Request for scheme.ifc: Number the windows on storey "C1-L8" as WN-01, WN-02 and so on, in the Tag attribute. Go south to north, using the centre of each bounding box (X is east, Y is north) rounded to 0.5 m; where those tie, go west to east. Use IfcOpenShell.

First a look at what the model holds.

```python
import ifcopenshell
import ifcopenshell.util.element
import ifcopenshell.util.placement

model = ifcopenshell.open("scheme.ifc")
print(model.schema)
storey = next(s for s in model.by_type("IfcBuildingStorey") if s.Name == "C1-L8")
windows = [e for e in ifcopenshell.util.element.get_decomposition(storey) if e.is_a("IfcWindow")]
for e in sorted(windows, key=lambda e: e.id()):
    origin = ifcopenshell.util.placement.get_local_placement(e.ObjectPlacement)[:3, 3]
    print(e.id(), e.Tag, e.Name, origin.round(2) + 0.0, sep=" | ")
```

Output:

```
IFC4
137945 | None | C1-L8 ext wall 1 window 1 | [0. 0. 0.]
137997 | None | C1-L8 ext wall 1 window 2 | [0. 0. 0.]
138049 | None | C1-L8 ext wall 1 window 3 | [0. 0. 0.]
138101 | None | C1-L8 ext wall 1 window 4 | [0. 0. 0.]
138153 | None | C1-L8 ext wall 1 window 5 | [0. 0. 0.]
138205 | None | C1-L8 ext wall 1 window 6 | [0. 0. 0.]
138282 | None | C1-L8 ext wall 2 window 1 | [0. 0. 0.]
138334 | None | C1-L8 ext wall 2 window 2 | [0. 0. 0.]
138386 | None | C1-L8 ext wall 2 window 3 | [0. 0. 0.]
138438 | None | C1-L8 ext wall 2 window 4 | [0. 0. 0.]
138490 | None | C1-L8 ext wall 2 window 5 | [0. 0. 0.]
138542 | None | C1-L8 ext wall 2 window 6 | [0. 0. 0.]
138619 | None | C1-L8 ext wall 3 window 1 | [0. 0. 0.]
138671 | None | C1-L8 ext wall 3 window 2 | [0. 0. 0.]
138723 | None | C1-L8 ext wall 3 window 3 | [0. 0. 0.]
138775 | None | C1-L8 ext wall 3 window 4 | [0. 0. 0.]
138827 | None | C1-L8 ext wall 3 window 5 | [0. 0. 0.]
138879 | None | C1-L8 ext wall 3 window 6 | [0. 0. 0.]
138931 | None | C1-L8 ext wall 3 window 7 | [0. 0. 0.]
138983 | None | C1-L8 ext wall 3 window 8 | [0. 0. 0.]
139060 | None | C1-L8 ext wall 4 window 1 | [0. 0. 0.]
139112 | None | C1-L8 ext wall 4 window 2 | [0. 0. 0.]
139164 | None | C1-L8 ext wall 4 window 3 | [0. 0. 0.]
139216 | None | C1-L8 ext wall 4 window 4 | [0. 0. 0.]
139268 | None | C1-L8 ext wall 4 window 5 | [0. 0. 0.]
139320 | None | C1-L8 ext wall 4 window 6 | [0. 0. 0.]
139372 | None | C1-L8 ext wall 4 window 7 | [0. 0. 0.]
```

```python
import ifcopenshell
import ifcopenshell.geom
import ifcopenshell.util.element
import ifcopenshell.util.shape

model = ifcopenshell.open("scheme.ifc")
settings = ifcopenshell.geom.settings()
settings.set("use-world-coords", True)


def centre(element):
    shape = ifcopenshell.geom.create_shape(settings, element)
    return ifcopenshell.util.shape.get_bbox_centroid(shape.geometry)


storey = next(s for s in model.by_type("IfcBuildingStorey") if s.Name == "C1-L8")
windows = [e for e in ifcopenshell.util.element.get_decomposition(storey) if e.is_a("IfcWindow")]

# Insertion points can sit at a corner or the storey origin, so sort by the geometry (in metres).
centres = {e: centre(e) for e in windows}
windows.sort(key=lambda e: (round(centres[e][1] / 0.5), centres[e][0]))

for i, e in enumerate(windows, start=1):
    number = f"WN-{i:02d}"
    e.Tag = number
    print(e.id(), number)

model.write("scheme_v2.ifc")
```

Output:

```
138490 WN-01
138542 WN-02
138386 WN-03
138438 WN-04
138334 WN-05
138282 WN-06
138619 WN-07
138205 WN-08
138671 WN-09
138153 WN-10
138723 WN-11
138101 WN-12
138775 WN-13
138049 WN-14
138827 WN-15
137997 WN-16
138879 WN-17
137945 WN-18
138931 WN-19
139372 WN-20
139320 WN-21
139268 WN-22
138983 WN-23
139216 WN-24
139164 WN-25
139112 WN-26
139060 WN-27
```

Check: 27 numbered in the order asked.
